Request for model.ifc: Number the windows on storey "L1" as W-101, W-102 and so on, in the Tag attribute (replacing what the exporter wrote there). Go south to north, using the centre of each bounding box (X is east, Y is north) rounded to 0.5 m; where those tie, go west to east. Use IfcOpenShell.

First a look at what the model holds.

```python
import ifcopenshell
import ifcopenshell.util.element
import ifcopenshell.util.placement

model = ifcopenshell.open("model.ifc")
print(model.schema)
storey = next(s for s in model.by_type("IfcBuildingStorey") if s.Name == "L1")
windows = [e for e in ifcopenshell.util.element.get_decomposition(storey) if e.is_a("IfcWindow")]
for e in sorted(windows, key=lambda e: e.id()):
    origin = ifcopenshell.util.placement.get_local_placement(e.ObjectPlacement)[:3, 3]
    print(e.id(), e.Tag, e.Name, origin.round(2) + 0.0, sep=" | ")
```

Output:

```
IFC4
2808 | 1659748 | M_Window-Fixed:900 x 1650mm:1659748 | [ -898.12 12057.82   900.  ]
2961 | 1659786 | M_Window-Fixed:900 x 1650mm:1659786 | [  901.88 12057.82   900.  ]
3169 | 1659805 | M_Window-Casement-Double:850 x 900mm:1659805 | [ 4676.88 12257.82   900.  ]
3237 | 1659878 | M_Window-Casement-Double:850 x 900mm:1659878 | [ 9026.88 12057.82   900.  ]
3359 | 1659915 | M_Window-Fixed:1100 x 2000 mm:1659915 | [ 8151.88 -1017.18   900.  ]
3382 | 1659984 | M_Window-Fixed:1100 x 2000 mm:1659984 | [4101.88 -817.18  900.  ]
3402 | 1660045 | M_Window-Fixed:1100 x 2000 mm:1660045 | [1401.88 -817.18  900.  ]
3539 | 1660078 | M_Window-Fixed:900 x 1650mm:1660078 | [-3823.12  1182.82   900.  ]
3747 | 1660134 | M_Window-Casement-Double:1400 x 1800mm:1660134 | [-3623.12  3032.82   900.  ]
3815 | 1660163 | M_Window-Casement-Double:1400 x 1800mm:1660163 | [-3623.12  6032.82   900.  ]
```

```python
import ifcopenshell
import ifcopenshell.geom
import ifcopenshell.util.element
import ifcopenshell.util.shape

model = ifcopenshell.open("model.ifc")
settings = ifcopenshell.geom.settings()
settings.set("use-world-coords", True)


def centre(element):
    shape = ifcopenshell.geom.create_shape(settings, element)
    return ifcopenshell.util.shape.get_bbox_centroid(shape.geometry)


storey = next(s for s in model.by_type("IfcBuildingStorey") if s.Name == "L1")
windows = [e for e in ifcopenshell.util.element.get_decomposition(storey) if e.is_a("IfcWindow")]

# Insertion points can sit at a corner or the storey origin, so sort by the geometry (in metres).
centres = {e: centre(e) for e in windows}
windows.sort(key=lambda e: (round(centres[e][1] / 0.5), centres[e][0]))

for i, e in enumerate(windows, start=1):
    number = f"W-1{i:02d}"
    e.Tag = number
    print(e.id(), number)

model.write("model_edited.ifc")
```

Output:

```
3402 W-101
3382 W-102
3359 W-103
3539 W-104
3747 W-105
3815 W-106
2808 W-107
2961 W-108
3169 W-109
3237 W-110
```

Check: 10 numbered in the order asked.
